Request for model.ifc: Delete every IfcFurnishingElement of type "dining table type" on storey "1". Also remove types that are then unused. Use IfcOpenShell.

First a look at what the model holds.

```python
import ifcopenshell
import ifcopenshell.util.element

model = ifcopenshell.open("model.ifc")
print(model.schema)
storey = next(s for s in model.by_type("IfcBuildingStorey") if s.Name == "1")
furniture = [e for e in ifcopenshell.util.element.get_decomposition(storey) if e.is_a("IfcFurnishingElement")]
seen = {}
for e in furniture:
    element_type = ifcopenshell.util.element.get_type(e)
    name = element_type.Name if element_type not in (None, e) else None
    seen[name] = seen.get(name, 0) + 1
for name, count in sorted(seen.items(), key=str):
    print(count, "x", name)
```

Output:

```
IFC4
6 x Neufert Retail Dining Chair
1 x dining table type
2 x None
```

```python
import ifcopenshell
import ifcopenshell.api.root
import ifcopenshell.util.element

model = ifcopenshell.open("model.ifc")

storey = next(s for s in model.by_type("IfcBuildingStorey") if s.Name == "1")
furniture = [e for e in ifcopenshell.util.element.get_decomposition(storey) if e.is_a("IfcFurnishingElement")]
targets = [e for e in furniture if (t := ifcopenshell.util.element.get_type(e)) not in (None, e) and t.Name == "dining table type"]
types = {ifcopenshell.util.element.get_type(e) for e in targets} - {None, *targets}

for e in targets:
    ifcopenshell.api.root.remove_product(model, product=e)
print(len(targets), "removed")

unused = [t for t in types if not ifcopenshell.util.element.get_types(t)]
for t in unused:
    ifcopenshell.api.root.remove_product(model, product=t)
print(len(unused), "unused types removed")

model.write("model_updated.ifc")
```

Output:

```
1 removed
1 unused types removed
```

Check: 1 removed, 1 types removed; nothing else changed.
